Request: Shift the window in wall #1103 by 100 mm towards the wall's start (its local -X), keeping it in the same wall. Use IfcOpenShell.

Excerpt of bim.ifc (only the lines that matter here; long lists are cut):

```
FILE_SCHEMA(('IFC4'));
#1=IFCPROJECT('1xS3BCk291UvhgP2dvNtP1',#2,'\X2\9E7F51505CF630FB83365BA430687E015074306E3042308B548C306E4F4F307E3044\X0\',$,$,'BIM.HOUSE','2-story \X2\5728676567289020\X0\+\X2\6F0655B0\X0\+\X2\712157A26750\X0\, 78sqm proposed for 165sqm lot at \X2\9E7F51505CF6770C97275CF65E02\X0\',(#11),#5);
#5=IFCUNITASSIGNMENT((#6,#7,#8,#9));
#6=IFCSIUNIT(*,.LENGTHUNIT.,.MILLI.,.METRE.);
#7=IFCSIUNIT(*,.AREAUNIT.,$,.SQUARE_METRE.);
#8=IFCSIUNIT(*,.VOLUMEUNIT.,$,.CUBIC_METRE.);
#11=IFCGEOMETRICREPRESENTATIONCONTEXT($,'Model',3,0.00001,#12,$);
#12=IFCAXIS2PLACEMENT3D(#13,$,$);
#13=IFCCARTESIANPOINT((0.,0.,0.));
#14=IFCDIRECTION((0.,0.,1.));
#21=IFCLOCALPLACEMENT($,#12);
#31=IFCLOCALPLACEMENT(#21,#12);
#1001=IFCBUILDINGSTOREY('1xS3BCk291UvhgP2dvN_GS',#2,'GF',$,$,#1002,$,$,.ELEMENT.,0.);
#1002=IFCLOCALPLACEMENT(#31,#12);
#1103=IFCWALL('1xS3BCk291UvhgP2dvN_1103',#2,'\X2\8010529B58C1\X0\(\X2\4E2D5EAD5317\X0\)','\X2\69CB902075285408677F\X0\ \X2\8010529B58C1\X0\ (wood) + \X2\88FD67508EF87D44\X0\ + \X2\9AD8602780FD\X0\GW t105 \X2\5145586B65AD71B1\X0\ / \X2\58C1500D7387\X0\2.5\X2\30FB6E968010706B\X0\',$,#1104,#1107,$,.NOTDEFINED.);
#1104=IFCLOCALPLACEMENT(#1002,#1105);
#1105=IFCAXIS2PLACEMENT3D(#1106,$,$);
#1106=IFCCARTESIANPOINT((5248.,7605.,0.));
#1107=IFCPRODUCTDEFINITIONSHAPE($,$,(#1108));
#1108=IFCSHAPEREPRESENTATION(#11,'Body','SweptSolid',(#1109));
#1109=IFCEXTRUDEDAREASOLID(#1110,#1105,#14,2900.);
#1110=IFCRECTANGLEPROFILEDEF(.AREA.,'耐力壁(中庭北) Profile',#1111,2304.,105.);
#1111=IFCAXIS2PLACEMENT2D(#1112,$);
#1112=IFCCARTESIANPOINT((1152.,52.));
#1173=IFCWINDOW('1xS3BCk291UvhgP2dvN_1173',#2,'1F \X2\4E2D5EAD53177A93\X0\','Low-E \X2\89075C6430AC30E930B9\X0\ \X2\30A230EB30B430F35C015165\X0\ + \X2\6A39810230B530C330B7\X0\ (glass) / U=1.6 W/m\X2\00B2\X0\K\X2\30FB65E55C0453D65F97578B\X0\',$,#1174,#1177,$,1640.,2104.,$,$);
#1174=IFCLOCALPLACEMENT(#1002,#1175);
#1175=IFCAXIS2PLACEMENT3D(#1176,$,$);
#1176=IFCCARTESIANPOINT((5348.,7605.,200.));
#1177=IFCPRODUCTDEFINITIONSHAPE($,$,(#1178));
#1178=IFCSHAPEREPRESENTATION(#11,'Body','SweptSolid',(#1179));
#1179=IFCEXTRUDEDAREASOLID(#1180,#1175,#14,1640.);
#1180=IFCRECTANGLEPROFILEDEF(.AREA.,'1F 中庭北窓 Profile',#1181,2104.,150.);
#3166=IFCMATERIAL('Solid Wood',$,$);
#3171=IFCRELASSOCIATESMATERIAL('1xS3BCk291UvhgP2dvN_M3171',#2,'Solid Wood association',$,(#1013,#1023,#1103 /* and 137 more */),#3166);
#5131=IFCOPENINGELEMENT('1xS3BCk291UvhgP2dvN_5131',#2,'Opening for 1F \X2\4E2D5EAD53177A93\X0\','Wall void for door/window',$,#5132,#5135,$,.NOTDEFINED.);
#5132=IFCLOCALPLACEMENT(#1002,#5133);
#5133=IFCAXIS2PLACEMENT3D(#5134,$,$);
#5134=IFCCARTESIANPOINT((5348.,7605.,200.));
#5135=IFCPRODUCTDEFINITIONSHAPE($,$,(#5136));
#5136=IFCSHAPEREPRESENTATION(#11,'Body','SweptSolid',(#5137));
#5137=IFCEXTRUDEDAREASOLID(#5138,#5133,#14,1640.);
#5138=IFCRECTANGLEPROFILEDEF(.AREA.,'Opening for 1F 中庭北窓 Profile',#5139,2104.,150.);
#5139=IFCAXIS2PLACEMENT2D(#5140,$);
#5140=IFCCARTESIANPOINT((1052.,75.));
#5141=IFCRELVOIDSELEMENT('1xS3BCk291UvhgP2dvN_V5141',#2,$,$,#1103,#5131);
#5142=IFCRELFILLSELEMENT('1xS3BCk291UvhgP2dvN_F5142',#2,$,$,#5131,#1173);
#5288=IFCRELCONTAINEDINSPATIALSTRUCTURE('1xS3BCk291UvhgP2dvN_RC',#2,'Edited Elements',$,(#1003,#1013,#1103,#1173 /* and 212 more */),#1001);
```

```python
import ifcopenshell
import ifcopenshell.api.geometry
import ifcopenshell.util.placement
import ifcopenshell.util.unit

model = ifcopenshell.open("bim.ifc")
unit_scale = ifcopenshell.util.unit.calculate_unit_scale(model)

window = model.by_guid("1xS3BCk291UvhgP2dvN_1173")
opening = window.FillsVoids[0].RelatingOpeningElement
wall = opening.VoidsElements[0].RelatingBuildingElement

wall_matrix = ifcopenshell.util.placement.get_local_placement(wall.ObjectPlacement)
shift = wall_matrix[:3, 0] * -0.1 / unit_scale
before = ifcopenshell.util.placement.get_local_placement(window.ObjectPlacement)[:3, 3].copy()

# The window is not placed relative to its opening, so move both.
for product in (opening, window):
    matrix = ifcopenshell.util.placement.get_local_placement(product.ObjectPlacement)
    matrix[:3, 3] += shift
    ifcopenshell.api.geometry.edit_object_placement(model, product=product, matrix=matrix, is_si=False)

after = ifcopenshell.util.placement.get_local_placement(window.ObjectPlacement)[:3, 3]
print("window moved by", (after - before).round(3) + 0.0)

model.write("bim_updated.ifc")
```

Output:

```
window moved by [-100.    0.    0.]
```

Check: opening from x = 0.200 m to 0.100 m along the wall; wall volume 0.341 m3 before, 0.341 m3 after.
